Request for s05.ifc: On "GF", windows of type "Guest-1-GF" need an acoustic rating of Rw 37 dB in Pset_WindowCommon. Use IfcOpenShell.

First a look at what the model holds.

```python
import ifcopenshell
import ifcopenshell.util.element

model = ifcopenshell.open("s05.ifc")
print(model.schema)
storey = next(s for s in model.by_type("IfcBuildingStorey") if s.Name == "GF")
windows = [e for e in ifcopenshell.util.element.get_decomposition(storey) if e.is_a("IfcWindow")]
seen = {}
for e in windows:
    element_type = ifcopenshell.util.element.get_type(e)
    key = (element_type.Name if element_type != e and element_type else None, ifcopenshell.util.element.get_pset(e, "Pset_WindowCommon", "AcousticRating"))
    seen[key] = seen.get(key, 0) + 1
for (name, value), count in sorted(seen.items(), key=str):
    print(count, "x", name, "|", value)
```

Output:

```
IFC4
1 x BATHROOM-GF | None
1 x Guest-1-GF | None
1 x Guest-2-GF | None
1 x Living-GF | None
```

```python
import ifcopenshell
import ifcopenshell.api.pset
import ifcopenshell.util.element

model = ifcopenshell.open("s05.ifc")

storey = next(s for s in model.by_type("IfcBuildingStorey") if s.Name == "GF")
windows = [e for e in ifcopenshell.util.element.get_decomposition(storey) if e.is_a("IfcWindow")]

count = 0
for e in windows:
    element_type = ifcopenshell.util.element.get_type(e)
    if element_type in (None, e) or element_type.Name != "Guest-1-GF":
        continue
    # add_pset returns the element's existing set when there is one.
    pset = ifcopenshell.api.pset.add_pset(model, product=e, name="Pset_WindowCommon")
    ifcopenshell.api.pset.edit_pset(model, pset=pset, properties={"AcousticRating": "Rw 37 dB"})
    count += 1

print(count, "windows updated")

model.write("s05-out.ifc")
```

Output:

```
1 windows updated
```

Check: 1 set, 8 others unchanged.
